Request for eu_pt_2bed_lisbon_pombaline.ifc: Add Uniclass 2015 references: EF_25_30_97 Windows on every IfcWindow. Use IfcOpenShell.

First a look at what the model holds.

```python
import ifcopenshell

model = ifcopenshell.open("eu_pt_2bed_lisbon_pombaline.ifc")
print(model.schema)
print("classifications:", [c.Name for c in model.by_type("IfcClassification")])
for ifc_class in ("IfcDoor", "IfcRoof", "IfcStair", "IfcWall", "IfcWindow"):
    print(ifc_class, len(model.by_type(ifc_class)))
```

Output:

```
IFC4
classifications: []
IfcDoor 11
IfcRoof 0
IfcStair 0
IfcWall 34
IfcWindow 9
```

```python
import ifcopenshell
import ifcopenshell.api.classification

model = ifcopenshell.open("eu_pt_2bed_lisbon_pombaline.ifc")

system = ifcopenshell.api.classification.add_classification(model, classification="Uniclass 2015")

codes = {
    "IfcWindow": ("EF_25_30_97", "Windows"),
}
for ifc_class, (code, name) in codes.items():
    products = model.by_type(ifc_class)
    ifcopenshell.api.classification.add_reference(
        model, products=products, classification=system, identification=code, name=name
    )
    print(code, len(products))

model.write("eu_pt_2bed_lisbon_pombaline_edited.ifc")
```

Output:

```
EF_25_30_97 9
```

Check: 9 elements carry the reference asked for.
